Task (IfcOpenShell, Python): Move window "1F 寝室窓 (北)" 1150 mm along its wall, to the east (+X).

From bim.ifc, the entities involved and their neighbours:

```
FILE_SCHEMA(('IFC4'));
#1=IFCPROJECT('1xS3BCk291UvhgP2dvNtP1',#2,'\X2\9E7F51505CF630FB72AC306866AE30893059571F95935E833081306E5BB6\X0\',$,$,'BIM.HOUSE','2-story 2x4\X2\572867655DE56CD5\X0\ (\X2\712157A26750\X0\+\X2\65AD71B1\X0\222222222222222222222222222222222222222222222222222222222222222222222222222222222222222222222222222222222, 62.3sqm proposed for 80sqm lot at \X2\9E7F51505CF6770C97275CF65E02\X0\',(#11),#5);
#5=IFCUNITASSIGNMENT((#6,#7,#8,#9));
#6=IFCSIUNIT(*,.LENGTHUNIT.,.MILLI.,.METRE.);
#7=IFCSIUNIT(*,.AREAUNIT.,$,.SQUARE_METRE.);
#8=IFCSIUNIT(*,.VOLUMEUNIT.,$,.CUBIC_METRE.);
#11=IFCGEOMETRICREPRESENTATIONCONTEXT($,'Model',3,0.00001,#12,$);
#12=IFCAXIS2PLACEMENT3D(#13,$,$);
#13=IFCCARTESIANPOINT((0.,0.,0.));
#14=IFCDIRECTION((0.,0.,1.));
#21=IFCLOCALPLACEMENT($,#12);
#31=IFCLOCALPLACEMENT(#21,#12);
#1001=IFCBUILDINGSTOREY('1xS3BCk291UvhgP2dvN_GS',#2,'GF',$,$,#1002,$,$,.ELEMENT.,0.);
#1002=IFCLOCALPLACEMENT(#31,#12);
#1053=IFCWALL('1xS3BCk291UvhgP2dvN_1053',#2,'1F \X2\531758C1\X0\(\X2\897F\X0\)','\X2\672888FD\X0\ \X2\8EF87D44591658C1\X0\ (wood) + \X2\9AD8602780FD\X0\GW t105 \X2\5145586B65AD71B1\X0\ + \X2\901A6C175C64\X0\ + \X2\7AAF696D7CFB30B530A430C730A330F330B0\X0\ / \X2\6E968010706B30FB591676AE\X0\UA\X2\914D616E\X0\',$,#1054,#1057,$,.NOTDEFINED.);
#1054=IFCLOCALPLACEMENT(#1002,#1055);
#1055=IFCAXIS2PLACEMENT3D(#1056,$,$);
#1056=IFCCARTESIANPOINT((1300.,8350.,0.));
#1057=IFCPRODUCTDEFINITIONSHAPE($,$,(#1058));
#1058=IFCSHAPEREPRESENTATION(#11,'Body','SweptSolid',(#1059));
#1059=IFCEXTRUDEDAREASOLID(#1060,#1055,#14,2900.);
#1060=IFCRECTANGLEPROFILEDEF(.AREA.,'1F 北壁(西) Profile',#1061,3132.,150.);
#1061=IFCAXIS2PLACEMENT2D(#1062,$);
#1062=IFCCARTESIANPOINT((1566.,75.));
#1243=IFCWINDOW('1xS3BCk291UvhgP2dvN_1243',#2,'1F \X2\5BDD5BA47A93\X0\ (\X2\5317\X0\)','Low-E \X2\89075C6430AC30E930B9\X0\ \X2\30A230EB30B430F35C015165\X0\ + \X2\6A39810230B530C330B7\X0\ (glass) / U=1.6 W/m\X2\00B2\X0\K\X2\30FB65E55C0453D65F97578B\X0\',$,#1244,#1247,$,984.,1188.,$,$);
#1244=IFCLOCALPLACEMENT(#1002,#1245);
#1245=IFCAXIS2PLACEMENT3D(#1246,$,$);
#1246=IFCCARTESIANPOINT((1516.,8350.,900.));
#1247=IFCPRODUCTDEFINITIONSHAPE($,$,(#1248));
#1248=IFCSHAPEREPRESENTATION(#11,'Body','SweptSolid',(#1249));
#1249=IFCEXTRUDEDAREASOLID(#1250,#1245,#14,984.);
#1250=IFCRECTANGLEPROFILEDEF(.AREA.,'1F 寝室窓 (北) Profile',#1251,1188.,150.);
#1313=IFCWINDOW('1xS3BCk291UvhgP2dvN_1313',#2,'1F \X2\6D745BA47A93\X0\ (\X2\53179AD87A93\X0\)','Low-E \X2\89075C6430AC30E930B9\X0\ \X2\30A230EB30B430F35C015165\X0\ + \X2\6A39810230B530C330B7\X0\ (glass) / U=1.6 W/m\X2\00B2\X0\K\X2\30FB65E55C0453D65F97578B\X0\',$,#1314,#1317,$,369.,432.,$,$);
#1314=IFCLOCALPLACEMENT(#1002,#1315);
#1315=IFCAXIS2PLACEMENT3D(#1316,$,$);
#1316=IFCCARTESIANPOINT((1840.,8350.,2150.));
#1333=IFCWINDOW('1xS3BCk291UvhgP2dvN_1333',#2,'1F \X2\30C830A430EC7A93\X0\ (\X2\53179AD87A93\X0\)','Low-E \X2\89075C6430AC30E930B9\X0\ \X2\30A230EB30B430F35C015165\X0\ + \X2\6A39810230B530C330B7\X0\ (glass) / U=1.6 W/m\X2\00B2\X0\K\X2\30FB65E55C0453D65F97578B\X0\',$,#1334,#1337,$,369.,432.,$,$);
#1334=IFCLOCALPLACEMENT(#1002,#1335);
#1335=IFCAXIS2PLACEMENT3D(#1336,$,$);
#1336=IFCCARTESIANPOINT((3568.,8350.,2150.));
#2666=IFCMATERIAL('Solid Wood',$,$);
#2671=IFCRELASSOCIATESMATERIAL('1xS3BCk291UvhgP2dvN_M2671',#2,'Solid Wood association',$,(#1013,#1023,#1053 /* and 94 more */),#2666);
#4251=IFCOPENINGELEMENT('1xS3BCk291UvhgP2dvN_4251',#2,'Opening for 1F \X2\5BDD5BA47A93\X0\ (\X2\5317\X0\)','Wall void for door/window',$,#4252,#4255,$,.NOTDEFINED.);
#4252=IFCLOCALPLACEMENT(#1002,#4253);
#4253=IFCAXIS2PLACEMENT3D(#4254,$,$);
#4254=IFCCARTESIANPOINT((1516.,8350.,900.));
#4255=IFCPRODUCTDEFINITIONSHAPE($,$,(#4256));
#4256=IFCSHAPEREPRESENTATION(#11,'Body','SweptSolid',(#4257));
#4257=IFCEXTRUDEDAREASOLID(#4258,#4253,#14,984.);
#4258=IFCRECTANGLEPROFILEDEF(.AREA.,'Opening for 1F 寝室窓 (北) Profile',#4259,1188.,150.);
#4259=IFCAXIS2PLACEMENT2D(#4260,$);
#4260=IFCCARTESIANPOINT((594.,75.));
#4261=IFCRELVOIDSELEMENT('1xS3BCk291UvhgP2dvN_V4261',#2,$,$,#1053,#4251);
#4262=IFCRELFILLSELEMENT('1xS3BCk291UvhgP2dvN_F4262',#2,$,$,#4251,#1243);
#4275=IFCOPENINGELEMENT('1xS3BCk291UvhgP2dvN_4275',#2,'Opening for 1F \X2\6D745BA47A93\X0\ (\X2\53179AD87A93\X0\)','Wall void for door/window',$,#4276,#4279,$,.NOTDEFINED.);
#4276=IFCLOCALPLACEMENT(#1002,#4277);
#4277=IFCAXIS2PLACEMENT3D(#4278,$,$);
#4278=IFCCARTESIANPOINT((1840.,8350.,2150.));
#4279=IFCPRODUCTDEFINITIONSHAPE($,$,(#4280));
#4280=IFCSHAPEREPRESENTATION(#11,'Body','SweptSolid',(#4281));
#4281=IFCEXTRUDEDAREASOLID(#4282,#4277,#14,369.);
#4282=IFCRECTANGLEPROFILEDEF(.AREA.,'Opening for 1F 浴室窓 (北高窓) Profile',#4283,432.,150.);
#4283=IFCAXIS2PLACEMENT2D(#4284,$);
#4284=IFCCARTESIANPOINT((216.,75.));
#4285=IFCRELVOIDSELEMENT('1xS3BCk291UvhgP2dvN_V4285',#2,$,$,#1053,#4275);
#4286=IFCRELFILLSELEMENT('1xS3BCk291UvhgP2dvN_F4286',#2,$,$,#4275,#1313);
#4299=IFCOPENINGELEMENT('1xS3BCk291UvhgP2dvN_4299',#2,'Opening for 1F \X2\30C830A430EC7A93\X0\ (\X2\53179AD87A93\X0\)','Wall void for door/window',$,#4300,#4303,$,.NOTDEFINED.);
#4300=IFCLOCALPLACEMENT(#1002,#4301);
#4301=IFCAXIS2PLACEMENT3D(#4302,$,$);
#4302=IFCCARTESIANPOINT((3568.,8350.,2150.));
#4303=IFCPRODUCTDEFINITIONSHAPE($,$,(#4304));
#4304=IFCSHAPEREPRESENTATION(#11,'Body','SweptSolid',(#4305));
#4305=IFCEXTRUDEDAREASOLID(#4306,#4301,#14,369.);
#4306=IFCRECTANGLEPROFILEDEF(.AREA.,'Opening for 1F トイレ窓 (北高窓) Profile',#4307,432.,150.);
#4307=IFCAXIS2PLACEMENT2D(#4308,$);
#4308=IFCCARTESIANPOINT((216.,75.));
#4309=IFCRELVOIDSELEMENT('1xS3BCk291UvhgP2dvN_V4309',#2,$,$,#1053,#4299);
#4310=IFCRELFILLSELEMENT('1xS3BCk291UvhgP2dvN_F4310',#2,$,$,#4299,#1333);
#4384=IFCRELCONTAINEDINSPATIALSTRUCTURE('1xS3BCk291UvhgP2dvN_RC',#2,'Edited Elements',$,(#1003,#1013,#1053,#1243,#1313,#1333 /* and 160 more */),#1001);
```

```python
import ifcopenshell
import ifcopenshell.api.geometry
import ifcopenshell.util.placement

model = ifcopenshell.open("bim.ifc")

window = model.by_guid("1xS3BCk291UvhgP2dvN_1243")
opening = window.FillsVoids[0].RelatingOpeningElement
wall = opening.VoidsElements[0].RelatingBuildingElement

wall_matrix = ifcopenshell.util.placement.get_local_placement(wall.ObjectPlacement)
shift = wall_matrix[:3, 0] * 1150.0
before = ifcopenshell.util.placement.get_local_placement(window.ObjectPlacement)[:3, 3].copy()

# The window is not placed relative to its opening, so move both.
for product in (opening, window):
    matrix = ifcopenshell.util.placement.get_local_placement(product.ObjectPlacement)
    matrix[:3, 3] += shift
    ifcopenshell.api.geometry.edit_object_placement(model, product=product, matrix=matrix, is_si=False)

after = ifcopenshell.util.placement.get_local_placement(window.ObjectPlacement)[:3, 3]
print("window moved by", (after - before).round(3) + 0.0)

model.write("bim_updated.ifc")
```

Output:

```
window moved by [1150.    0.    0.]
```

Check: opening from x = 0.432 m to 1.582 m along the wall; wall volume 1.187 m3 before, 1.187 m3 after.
